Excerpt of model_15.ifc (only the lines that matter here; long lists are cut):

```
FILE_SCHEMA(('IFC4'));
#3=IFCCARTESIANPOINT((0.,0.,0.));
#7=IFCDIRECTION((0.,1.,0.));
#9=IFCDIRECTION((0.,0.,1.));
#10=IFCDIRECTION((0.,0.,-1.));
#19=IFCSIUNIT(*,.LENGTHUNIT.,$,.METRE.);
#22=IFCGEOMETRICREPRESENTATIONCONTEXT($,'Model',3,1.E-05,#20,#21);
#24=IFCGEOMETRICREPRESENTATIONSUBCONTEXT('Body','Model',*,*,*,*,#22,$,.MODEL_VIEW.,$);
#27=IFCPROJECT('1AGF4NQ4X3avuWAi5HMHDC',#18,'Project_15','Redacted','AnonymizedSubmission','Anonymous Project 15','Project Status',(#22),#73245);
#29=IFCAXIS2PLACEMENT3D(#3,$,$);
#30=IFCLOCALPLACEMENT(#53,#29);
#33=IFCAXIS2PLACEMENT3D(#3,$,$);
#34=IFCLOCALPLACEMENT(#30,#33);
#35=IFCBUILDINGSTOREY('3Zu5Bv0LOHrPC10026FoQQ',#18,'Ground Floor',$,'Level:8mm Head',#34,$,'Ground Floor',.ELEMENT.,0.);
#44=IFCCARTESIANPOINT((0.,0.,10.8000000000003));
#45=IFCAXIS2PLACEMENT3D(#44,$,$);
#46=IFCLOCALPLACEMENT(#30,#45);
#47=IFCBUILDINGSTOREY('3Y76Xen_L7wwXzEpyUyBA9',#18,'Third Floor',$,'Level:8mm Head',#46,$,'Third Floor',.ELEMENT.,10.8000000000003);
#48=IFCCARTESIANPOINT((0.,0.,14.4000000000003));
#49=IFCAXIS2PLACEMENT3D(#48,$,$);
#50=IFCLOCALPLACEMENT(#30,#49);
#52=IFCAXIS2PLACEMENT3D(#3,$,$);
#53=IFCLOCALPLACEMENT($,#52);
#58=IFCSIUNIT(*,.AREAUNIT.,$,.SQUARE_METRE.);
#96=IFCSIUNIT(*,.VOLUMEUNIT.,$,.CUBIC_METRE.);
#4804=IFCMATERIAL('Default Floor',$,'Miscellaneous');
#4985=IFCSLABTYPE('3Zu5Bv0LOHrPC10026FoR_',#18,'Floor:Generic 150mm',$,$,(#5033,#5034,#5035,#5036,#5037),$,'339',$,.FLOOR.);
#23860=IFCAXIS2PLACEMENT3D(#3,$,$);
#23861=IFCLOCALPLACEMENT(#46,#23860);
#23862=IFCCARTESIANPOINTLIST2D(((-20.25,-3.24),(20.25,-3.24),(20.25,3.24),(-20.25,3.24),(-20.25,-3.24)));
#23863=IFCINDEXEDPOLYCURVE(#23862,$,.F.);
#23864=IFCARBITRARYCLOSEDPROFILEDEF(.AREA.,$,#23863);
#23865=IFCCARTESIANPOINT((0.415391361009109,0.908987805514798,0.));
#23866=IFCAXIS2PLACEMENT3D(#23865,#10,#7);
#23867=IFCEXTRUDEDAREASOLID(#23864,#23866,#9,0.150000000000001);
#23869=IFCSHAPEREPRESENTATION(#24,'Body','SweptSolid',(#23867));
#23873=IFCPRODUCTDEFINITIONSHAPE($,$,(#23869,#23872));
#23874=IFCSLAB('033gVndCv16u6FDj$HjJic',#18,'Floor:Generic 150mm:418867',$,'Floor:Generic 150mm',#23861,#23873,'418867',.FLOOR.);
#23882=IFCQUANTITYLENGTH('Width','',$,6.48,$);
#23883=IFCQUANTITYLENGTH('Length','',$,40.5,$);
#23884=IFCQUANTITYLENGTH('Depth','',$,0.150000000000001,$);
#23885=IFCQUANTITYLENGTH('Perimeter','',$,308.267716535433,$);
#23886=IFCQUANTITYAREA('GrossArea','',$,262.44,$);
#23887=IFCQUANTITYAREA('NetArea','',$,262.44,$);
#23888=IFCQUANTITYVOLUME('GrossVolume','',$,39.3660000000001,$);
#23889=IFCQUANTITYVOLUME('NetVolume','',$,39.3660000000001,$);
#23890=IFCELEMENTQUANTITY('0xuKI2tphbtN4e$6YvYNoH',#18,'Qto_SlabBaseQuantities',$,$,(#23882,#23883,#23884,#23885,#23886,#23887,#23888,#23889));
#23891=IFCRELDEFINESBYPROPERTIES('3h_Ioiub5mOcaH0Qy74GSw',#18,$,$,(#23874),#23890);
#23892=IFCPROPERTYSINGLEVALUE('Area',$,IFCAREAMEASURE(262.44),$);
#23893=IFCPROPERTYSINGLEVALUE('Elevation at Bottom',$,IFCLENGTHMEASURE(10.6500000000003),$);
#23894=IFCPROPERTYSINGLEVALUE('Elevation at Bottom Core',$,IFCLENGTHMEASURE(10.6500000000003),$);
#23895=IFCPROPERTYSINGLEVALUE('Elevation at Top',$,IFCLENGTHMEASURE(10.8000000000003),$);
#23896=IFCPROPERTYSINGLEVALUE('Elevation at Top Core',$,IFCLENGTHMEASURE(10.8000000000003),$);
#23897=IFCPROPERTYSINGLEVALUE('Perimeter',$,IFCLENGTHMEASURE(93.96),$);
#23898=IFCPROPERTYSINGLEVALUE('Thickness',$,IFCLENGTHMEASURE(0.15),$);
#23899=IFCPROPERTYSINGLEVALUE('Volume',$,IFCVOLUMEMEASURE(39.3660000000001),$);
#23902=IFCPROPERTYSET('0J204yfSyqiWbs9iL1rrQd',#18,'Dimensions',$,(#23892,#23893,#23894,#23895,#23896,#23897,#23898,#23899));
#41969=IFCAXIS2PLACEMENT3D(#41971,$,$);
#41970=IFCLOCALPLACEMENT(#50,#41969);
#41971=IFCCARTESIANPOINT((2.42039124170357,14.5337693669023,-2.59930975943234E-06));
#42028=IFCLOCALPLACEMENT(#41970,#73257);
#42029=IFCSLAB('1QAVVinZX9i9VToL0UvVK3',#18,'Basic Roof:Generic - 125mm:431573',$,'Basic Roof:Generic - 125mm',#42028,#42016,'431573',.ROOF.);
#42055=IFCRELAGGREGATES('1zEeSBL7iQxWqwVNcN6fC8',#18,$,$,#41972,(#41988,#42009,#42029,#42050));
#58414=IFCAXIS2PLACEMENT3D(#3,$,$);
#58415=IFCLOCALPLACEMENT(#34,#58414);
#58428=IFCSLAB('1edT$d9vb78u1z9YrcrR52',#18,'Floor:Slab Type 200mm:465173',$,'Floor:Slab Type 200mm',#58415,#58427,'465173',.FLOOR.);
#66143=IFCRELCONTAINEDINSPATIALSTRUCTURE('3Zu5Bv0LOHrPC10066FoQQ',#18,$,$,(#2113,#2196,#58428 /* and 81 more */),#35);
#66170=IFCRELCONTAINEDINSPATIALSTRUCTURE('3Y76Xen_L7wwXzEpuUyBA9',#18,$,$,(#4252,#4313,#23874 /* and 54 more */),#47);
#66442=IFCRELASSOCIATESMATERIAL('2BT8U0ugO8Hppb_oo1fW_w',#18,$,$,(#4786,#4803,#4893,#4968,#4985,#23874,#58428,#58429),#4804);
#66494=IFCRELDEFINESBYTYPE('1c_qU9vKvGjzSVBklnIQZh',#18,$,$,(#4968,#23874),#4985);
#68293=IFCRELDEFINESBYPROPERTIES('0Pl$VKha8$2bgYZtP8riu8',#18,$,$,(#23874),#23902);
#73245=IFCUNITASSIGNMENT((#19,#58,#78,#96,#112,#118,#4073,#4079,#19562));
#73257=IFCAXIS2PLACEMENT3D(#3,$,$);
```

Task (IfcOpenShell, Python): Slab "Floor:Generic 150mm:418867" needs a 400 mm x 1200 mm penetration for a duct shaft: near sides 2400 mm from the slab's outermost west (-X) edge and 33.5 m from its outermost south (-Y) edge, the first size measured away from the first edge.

```python
import numpy as np
import ifcopenshell
import ifcopenshell.api.feature
import ifcopenshell.api.geometry
import ifcopenshell.api.pset
import ifcopenshell.api.root
import ifcopenshell.geom
import ifcopenshell.util.element
import ifcopenshell.util.placement
import ifcopenshell.util.representation
import ifcopenshell.util.shape
import ifcopenshell.util.unit

model = ifcopenshell.open("model_15.ifc")
unit_scale = ifcopenshell.util.unit.calculate_unit_scale(model)
area_scale = ifcopenshell.util.unit.calculate_unit_scale(model, "AREAUNIT")
volume_scale = ifcopenshell.util.unit.calculate_unit_scale(model, "VOLUMEUNIT")
settings = ifcopenshell.geom.settings()


def volume(element):
    """Net volume in cubic metres, openings subtracted."""
    shape = ifcopenshell.geom.create_shape(settings, element)
    return ifcopenshell.util.shape.get_volume(shape.geometry)


slab = model.by_guid("033gVndCv16u6FDj$HjJic")
before = volume(slab)

# Extent in the slab's own axes, in metres. The edges named are its -X and -Y sides.
slab_shape = ifcopenshell.geom.create_shape(settings, slab)
vertices = ifcopenshell.util.shape.get_vertices(slab_shape.geometry)
x_min, y_min, bottom = vertices.min(axis=0)
top = vertices[:, 2].max()

opening = ifcopenshell.api.root.create_entity(model, ifc_class="IfcOpeningElement", name="Duct shaft opening", predefined_type="OPENING")
context = ifcopenshell.util.representation.get_context(model, "Model", "Body", "MODEL_VIEW")
width, depth = 0.4, 1.2
outline = [(0.0, 0.0), (width, 0.0), (width, depth), (0.0, depth), (0.0, 0.0)]
# Overshoot both faces by 50 mm so the cut is clean.
shape = ifcopenshell.api.geometry.add_slab_representation(
    model, context=context, depth=top - bottom + 0.1, polyline=outline
)
ifcopenshell.api.geometry.assign_representation(model, product=opening, representation=shape)

matrix = ifcopenshell.util.placement.get_local_placement(slab.ObjectPlacement)
matrix[:, 3] = matrix @ np.append(np.array([x_min + 2.4, y_min + 33.5, bottom - 0.05]) / unit_scale, 1.0)
ifcopenshell.api.geometry.edit_object_placement(model, product=opening, matrix=matrix, is_si=False)
ifcopenshell.api.feature.add_feature(model, feature=opening, element=slab)

after = volume(slab)

# Update the slab's stored quantities.
qto = model.by_id(ifcopenshell.util.element.get_pset(slab, "Qto_SlabBaseQuantities", should_inherit=False)["id"])
ifcopenshell.api.pset.edit_qto(model, qto=qto, properties={
    "NetArea": after / (top - bottom) / area_scale,
    "NetVolume": after / volume_scale,
})
pset = model.by_id(ifcopenshell.util.element.get_pset(slab, "Dimensions", should_inherit=False)["id"])
ifcopenshell.api.pset.edit_pset(model, pset=pset, properties={
    "Area": model.create_entity("IfcAreaMeasure", after / (top - bottom) / area_scale),
    "Volume": model.create_entity("IfcVolumeMeasure", after / volume_scale),
})

print(f"slab volume {before:.3f} -> {after:.3f} m3")

model.write("model_15_updated.ifc")
```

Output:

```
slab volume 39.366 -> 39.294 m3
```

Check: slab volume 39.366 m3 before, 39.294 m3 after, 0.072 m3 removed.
